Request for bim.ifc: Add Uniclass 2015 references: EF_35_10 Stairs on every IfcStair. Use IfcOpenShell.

First a look at what the model holds.

```python
import ifcopenshell

model = ifcopenshell.open("bim.ifc")
print(model.schema)
print("classifications:", [c.Name for c in model.by_type("IfcClassification")])
for ifc_class in ("IfcDoor", "IfcRoof", "IfcStair", "IfcWall", "IfcWindow"):
    print(ifc_class, len(model.by_type(ifc_class)))
```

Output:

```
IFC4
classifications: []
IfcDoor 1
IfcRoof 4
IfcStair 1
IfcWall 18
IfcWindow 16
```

```python
import ifcopenshell
import ifcopenshell.api.classification

model = ifcopenshell.open("bim.ifc")

system = ifcopenshell.api.classification.add_classification(model, classification="Uniclass 2015")

codes = {
    "IfcStair": ("EF_35_10", "Stairs"),
}
for ifc_class, (code, name) in codes.items():
    products = model.by_type(ifc_class)
    ifcopenshell.api.classification.add_reference(
        model, products=products, classification=system, identification=code, name=name
    )
    print(code, len(products))

model.write("bim_rev.ifc")
```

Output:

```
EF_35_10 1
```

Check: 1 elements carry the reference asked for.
